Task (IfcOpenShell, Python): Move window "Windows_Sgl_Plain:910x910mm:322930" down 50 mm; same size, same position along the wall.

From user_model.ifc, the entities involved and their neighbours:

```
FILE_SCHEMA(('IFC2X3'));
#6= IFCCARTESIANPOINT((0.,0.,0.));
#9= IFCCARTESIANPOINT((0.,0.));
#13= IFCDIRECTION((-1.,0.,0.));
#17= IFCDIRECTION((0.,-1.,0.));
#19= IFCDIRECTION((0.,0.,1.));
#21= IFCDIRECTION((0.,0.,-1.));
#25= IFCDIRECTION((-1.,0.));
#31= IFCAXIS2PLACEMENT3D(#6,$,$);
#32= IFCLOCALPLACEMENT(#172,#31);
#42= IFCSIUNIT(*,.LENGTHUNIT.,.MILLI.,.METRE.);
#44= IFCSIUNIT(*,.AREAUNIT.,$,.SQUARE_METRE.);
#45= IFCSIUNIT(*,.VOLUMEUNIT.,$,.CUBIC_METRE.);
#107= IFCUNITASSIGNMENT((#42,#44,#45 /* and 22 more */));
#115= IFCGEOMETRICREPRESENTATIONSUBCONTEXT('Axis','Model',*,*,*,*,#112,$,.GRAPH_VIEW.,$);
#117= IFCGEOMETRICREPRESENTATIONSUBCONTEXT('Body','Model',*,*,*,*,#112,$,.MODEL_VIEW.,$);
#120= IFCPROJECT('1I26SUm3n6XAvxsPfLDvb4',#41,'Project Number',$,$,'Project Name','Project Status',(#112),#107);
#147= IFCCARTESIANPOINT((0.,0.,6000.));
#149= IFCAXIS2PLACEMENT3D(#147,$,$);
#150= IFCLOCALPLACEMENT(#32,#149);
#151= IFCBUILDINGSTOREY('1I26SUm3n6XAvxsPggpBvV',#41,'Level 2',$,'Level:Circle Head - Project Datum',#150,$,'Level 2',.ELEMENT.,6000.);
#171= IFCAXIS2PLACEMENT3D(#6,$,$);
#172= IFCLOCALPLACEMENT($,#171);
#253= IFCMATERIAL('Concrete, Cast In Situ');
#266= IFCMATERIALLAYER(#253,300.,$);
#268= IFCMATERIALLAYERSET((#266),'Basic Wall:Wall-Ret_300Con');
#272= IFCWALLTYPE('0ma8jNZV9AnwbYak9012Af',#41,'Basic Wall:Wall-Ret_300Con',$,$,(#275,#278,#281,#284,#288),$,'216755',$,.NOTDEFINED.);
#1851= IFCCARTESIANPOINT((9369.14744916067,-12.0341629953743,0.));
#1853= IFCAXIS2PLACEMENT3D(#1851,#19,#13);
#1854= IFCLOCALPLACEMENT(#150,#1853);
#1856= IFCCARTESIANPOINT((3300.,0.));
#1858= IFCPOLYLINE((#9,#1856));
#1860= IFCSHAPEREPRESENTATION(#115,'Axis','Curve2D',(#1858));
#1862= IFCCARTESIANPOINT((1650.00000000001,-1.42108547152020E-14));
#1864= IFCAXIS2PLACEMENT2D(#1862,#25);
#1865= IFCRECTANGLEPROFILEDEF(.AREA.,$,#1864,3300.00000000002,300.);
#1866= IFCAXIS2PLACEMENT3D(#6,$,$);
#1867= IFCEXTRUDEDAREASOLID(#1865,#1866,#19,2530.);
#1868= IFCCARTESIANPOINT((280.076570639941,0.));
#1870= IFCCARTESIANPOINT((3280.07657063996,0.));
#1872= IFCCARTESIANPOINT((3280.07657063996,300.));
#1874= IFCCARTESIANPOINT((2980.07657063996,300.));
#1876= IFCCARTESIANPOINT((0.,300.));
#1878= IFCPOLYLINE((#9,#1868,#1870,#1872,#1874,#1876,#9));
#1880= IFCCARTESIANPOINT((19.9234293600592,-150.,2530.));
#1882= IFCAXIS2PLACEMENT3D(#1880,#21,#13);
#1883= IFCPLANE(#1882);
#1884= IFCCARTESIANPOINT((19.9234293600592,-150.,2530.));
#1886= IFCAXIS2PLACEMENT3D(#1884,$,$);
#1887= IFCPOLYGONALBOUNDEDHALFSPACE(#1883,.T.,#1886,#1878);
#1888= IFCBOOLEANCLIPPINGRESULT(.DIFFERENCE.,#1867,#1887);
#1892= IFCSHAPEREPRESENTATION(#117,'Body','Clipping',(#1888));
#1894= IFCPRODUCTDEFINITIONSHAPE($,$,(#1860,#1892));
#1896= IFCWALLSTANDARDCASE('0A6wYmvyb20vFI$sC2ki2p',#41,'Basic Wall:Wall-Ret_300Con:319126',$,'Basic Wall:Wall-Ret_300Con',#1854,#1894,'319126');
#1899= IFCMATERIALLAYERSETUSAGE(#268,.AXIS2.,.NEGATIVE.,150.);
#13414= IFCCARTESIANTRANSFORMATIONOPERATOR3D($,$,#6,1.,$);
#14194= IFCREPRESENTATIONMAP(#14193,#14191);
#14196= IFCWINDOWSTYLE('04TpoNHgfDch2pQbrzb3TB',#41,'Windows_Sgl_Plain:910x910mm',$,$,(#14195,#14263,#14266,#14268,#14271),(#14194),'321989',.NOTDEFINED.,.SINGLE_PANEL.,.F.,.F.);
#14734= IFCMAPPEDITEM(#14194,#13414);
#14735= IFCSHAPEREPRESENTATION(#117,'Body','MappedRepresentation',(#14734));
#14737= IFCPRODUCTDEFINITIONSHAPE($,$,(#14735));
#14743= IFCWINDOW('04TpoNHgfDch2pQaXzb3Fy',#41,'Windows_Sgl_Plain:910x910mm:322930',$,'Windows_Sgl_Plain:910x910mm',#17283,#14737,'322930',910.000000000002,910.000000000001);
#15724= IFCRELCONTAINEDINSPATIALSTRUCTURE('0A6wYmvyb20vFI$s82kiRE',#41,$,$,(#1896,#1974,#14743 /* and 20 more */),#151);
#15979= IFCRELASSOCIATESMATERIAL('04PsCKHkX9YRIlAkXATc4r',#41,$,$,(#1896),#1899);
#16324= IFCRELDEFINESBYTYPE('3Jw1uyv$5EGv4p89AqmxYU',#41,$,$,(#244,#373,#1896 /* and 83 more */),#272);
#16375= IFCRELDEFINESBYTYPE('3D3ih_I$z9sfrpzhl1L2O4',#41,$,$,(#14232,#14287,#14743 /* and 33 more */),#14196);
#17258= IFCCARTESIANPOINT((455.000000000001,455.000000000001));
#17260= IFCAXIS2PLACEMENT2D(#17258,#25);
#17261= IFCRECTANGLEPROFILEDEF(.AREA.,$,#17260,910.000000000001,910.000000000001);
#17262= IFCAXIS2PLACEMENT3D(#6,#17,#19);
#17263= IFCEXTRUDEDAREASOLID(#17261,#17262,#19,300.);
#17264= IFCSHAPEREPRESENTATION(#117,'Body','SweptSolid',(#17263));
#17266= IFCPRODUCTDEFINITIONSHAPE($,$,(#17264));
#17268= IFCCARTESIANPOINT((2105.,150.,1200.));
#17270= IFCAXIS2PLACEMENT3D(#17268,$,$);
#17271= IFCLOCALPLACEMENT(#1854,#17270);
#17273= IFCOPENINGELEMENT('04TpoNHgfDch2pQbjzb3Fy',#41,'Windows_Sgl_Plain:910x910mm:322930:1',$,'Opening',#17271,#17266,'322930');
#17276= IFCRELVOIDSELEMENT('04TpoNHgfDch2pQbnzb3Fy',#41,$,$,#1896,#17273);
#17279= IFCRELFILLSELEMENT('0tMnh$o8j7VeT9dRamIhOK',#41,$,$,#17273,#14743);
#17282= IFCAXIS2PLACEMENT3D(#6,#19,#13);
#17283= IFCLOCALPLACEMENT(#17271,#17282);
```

```python
import numpy as np
import ifcopenshell
import ifcopenshell.api.geometry
import ifcopenshell.util.placement
import ifcopenshell.util.unit

model = ifcopenshell.open("user_model.ifc")
unit_scale = ifcopenshell.util.unit.calculate_unit_scale(model)

window = model.by_guid("04TpoNHgfDch2pQaXzb3Fy")
opening = window.FillsVoids[0].RelatingOpeningElement
dz = -0.05 / unit_scale

shift = np.array([0.0, 0.0, dz])
# The window is placed relative to its opening, so it follows when the opening moves.
matrix = ifcopenshell.util.placement.get_local_placement(opening.ObjectPlacement)
matrix[:3, 3] += shift
ifcopenshell.api.geometry.edit_object_placement(
    model, product=opening, matrix=matrix, is_si=False, should_transform_children=True
)

print(f"moved by {dz * unit_scale:+.3f} m")

model.write("user_model_v2.ifc")
```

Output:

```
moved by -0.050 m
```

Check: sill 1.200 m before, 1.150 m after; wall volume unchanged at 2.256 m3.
